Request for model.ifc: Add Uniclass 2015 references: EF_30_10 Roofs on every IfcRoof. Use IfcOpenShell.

First a look at what the model holds.

```python
import ifcopenshell

model = ifcopenshell.open("model.ifc")
print(model.schema)
print("classifications:", [c.Name for c in model.by_type("IfcClassification")])
for ifc_class in ("IfcDoor", "IfcRoof", "IfcStair", "IfcWall", "IfcWindow"):
    print(ifc_class, len(model.by_type(ifc_class)))
```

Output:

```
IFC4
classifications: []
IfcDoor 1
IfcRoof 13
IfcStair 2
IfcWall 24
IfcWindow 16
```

```python
import ifcopenshell
import ifcopenshell.api.classification

model = ifcopenshell.open("model.ifc")

system = ifcopenshell.api.classification.add_classification(model, classification="Uniclass 2015")

codes = {
    "IfcRoof": ("EF_30_10", "Roofs"),
}
for ifc_class, (code, name) in codes.items():
    products = model.by_type(ifc_class)
    ifcopenshell.api.classification.add_reference(
        model, products=products, classification=system, identification=code, name=name
    )
    print(code, len(products))

model.write("model-out.ifc")
```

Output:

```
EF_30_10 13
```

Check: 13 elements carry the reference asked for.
